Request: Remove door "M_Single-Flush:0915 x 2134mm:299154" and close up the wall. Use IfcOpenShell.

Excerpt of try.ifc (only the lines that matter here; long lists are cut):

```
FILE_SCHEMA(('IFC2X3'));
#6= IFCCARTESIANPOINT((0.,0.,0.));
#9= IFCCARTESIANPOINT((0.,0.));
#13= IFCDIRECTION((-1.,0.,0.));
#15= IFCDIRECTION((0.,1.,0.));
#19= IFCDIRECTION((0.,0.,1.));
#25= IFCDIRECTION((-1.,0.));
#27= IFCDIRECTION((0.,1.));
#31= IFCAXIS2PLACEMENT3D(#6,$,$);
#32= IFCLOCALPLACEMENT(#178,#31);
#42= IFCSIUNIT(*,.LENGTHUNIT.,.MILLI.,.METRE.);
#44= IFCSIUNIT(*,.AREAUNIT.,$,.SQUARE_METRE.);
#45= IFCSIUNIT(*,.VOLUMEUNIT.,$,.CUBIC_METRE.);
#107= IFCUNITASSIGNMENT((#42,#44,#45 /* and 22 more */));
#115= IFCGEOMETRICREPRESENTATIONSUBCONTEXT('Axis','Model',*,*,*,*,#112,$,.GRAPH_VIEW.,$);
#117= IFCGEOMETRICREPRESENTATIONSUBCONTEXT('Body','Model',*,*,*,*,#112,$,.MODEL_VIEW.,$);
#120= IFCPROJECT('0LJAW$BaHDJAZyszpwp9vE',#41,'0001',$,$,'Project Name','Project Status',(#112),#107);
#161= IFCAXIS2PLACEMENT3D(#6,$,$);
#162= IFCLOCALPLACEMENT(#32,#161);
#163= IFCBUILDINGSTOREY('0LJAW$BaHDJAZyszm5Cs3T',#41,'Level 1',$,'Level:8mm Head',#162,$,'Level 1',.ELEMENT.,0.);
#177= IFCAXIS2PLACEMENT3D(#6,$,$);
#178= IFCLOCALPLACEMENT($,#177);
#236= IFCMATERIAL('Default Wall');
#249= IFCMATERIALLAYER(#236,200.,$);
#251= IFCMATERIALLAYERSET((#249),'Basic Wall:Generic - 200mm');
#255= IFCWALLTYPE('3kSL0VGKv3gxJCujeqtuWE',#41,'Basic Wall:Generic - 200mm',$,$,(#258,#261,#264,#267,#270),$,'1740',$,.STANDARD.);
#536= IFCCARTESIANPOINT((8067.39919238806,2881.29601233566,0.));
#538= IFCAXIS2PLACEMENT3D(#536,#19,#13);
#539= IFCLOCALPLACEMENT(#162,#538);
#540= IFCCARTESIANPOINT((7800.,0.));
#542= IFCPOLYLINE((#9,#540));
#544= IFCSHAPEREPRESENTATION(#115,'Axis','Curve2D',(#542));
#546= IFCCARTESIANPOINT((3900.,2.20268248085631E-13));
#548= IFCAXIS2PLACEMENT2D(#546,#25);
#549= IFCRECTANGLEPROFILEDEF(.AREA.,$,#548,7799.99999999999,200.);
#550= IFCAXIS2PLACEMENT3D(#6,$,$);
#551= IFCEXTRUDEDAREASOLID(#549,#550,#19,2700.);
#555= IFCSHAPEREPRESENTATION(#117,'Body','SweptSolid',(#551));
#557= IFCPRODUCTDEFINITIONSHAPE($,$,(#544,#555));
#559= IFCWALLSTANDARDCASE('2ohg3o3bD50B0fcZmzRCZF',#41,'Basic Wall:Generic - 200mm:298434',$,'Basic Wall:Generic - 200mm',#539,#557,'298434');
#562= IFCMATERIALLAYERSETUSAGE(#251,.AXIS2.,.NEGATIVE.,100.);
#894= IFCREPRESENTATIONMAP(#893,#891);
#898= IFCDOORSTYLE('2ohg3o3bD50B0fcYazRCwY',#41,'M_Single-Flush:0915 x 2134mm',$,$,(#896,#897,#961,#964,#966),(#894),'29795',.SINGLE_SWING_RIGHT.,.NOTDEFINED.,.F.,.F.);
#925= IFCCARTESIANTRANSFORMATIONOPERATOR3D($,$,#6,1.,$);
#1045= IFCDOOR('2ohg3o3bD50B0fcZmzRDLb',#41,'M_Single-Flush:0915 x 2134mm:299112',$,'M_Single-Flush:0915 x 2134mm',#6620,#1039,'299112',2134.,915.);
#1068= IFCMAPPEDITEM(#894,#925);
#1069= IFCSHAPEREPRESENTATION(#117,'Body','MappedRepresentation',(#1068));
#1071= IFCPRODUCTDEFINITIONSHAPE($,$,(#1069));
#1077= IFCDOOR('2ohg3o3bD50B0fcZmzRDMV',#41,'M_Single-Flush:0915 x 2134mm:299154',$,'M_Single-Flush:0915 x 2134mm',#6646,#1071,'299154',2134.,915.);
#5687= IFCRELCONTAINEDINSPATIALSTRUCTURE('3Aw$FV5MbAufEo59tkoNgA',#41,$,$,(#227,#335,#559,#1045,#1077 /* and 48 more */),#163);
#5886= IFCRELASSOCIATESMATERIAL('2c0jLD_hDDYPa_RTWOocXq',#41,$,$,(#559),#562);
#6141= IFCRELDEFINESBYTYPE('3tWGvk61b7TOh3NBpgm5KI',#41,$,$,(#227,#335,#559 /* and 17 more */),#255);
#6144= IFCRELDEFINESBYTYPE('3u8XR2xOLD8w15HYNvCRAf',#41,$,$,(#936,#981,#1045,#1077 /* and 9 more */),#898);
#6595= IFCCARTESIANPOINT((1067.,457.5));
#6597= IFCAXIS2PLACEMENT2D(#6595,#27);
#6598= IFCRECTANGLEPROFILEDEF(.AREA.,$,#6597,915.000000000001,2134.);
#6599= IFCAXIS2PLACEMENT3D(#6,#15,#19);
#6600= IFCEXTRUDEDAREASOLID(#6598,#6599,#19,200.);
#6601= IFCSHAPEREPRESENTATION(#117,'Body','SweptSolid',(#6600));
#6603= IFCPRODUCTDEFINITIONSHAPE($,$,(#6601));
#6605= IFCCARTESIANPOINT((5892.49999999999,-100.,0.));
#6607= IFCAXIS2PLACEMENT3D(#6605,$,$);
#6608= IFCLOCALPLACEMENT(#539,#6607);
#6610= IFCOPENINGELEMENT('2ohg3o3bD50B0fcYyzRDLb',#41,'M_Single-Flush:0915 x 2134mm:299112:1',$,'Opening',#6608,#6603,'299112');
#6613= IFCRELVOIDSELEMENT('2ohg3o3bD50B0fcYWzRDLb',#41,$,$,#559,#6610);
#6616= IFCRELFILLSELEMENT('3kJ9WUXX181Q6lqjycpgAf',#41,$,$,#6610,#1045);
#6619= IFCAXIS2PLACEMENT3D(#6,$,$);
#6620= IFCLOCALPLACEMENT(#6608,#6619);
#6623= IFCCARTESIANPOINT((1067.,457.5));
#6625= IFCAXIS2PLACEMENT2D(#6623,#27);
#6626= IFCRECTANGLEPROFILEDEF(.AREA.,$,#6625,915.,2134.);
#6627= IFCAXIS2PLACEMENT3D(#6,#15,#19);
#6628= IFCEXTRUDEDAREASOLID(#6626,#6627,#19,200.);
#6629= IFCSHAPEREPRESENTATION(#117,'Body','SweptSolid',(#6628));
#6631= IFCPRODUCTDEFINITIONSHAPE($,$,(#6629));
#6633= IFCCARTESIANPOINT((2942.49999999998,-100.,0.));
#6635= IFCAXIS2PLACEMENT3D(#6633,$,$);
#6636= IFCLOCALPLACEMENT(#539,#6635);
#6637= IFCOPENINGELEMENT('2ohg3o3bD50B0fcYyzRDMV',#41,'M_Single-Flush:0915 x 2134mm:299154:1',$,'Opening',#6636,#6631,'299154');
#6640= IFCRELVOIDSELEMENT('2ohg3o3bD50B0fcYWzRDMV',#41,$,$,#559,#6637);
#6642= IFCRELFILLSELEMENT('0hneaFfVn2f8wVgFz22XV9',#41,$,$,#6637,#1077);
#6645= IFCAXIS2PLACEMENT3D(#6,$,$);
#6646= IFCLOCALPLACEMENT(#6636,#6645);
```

```python
import ifcopenshell
import ifcopenshell.api.feature
import ifcopenshell.api.root
import ifcopenshell.geom
import ifcopenshell.util.shape

model = ifcopenshell.open("try.ifc")
settings = ifcopenshell.geom.settings()


def volume(element):
    """Net volume in cubic metres, openings subtracted."""
    shape = ifcopenshell.geom.create_shape(settings, element)
    return ifcopenshell.util.shape.get_volume(shape.geometry)


door = model.by_guid("2ohg3o3bD50B0fcZmzRDMV")
opening = door.FillsVoids[0].RelatingOpeningElement
wall = opening.VoidsElements[0].RelatingBuildingElement
before = volume(wall)

ifcopenshell.api.root.remove_product(model, product=door)
ifcopenshell.api.feature.remove_feature(model, feature=opening)

after = volume(wall)

print(f"wall volume {before:.3f} -> {after:.3f} m3")

model.write("try_updated.ifc")
```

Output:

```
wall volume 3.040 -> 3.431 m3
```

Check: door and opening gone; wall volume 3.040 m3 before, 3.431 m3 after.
